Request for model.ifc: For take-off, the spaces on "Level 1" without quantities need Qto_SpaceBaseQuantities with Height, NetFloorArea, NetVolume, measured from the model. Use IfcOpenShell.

First a look at what the model holds.

```python
import ifcopenshell
import ifcopenshell.util.element
import ifcopenshell.util.unit

model = ifcopenshell.open("model.ifc")
print(model.schema)
for unit_type in ("LENGTHUNIT", "AREAUNIT", "VOLUMEUNIT"):
    print(unit_type, ifcopenshell.util.unit.calculate_unit_scale(model, unit_type))
storey = next(s for s in model.by_type("IfcBuildingStorey") if s.Name == "Level 1")
spaces = [e for e in ifcopenshell.util.element.get_decomposition(storey) if e.is_a("IfcSpace")]
for e in sorted(spaces, key=lambda e: e.id()):
    print(e.id(), e.is_a(), e.Name, list(ifcopenshell.util.element.get_psets(e, qtos_only=True)), sep=" | ")
```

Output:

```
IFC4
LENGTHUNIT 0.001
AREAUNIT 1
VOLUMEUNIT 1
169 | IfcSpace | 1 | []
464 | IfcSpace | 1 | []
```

```python
import ifcopenshell
import ifcopenshell.api.pset
import ifcopenshell.geom
import ifcopenshell.util.element
import ifcopenshell.util.shape
import ifcopenshell.util.unit

model = ifcopenshell.open("model.ifc")
unit_scale = ifcopenshell.util.unit.calculate_unit_scale(model)
area_scale = ifcopenshell.util.unit.calculate_unit_scale(model, "AREAUNIT")
volume_scale = ifcopenshell.util.unit.calculate_unit_scale(model, "VOLUMEUNIT")
settings = ifcopenshell.geom.settings()

storey = next(s for s in model.by_type("IfcBuildingStorey") if s.Name == "Level 1")
spaces = [e for e in ifcopenshell.util.element.get_decomposition(storey) if e.is_a("IfcSpace")]

for e in sorted(spaces, key=lambda e: e.id()):
    if ifcopenshell.util.element.get_psets(e, qtos_only=True, should_inherit=False):
        continue
    # Geometry comes back in metres, in the element's own axes.
    shape = ifcopenshell.geom.create_shape(settings, e)
    values = {
        "Height": ifcopenshell.util.shape.get_z(shape.geometry) / unit_scale,
        "NetFloorArea": ifcopenshell.util.shape.get_footprint_area(shape.geometry) / area_scale,
        "NetVolume": ifcopenshell.util.shape.get_volume(shape.geometry) / volume_scale,
    }
    qto = ifcopenshell.api.pset.add_qto(model, product=e, name="Qto_SpaceBaseQuantities")
    ifcopenshell.api.pset.edit_qto(model, qto=qto, properties=values)
    print(e.id(), {k: round(v, 3) for k, v in values.items()})

model.write("model_updated.ifc")
```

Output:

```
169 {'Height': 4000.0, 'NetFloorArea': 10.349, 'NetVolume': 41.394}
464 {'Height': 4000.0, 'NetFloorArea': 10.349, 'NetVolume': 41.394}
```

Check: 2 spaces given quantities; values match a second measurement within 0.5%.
